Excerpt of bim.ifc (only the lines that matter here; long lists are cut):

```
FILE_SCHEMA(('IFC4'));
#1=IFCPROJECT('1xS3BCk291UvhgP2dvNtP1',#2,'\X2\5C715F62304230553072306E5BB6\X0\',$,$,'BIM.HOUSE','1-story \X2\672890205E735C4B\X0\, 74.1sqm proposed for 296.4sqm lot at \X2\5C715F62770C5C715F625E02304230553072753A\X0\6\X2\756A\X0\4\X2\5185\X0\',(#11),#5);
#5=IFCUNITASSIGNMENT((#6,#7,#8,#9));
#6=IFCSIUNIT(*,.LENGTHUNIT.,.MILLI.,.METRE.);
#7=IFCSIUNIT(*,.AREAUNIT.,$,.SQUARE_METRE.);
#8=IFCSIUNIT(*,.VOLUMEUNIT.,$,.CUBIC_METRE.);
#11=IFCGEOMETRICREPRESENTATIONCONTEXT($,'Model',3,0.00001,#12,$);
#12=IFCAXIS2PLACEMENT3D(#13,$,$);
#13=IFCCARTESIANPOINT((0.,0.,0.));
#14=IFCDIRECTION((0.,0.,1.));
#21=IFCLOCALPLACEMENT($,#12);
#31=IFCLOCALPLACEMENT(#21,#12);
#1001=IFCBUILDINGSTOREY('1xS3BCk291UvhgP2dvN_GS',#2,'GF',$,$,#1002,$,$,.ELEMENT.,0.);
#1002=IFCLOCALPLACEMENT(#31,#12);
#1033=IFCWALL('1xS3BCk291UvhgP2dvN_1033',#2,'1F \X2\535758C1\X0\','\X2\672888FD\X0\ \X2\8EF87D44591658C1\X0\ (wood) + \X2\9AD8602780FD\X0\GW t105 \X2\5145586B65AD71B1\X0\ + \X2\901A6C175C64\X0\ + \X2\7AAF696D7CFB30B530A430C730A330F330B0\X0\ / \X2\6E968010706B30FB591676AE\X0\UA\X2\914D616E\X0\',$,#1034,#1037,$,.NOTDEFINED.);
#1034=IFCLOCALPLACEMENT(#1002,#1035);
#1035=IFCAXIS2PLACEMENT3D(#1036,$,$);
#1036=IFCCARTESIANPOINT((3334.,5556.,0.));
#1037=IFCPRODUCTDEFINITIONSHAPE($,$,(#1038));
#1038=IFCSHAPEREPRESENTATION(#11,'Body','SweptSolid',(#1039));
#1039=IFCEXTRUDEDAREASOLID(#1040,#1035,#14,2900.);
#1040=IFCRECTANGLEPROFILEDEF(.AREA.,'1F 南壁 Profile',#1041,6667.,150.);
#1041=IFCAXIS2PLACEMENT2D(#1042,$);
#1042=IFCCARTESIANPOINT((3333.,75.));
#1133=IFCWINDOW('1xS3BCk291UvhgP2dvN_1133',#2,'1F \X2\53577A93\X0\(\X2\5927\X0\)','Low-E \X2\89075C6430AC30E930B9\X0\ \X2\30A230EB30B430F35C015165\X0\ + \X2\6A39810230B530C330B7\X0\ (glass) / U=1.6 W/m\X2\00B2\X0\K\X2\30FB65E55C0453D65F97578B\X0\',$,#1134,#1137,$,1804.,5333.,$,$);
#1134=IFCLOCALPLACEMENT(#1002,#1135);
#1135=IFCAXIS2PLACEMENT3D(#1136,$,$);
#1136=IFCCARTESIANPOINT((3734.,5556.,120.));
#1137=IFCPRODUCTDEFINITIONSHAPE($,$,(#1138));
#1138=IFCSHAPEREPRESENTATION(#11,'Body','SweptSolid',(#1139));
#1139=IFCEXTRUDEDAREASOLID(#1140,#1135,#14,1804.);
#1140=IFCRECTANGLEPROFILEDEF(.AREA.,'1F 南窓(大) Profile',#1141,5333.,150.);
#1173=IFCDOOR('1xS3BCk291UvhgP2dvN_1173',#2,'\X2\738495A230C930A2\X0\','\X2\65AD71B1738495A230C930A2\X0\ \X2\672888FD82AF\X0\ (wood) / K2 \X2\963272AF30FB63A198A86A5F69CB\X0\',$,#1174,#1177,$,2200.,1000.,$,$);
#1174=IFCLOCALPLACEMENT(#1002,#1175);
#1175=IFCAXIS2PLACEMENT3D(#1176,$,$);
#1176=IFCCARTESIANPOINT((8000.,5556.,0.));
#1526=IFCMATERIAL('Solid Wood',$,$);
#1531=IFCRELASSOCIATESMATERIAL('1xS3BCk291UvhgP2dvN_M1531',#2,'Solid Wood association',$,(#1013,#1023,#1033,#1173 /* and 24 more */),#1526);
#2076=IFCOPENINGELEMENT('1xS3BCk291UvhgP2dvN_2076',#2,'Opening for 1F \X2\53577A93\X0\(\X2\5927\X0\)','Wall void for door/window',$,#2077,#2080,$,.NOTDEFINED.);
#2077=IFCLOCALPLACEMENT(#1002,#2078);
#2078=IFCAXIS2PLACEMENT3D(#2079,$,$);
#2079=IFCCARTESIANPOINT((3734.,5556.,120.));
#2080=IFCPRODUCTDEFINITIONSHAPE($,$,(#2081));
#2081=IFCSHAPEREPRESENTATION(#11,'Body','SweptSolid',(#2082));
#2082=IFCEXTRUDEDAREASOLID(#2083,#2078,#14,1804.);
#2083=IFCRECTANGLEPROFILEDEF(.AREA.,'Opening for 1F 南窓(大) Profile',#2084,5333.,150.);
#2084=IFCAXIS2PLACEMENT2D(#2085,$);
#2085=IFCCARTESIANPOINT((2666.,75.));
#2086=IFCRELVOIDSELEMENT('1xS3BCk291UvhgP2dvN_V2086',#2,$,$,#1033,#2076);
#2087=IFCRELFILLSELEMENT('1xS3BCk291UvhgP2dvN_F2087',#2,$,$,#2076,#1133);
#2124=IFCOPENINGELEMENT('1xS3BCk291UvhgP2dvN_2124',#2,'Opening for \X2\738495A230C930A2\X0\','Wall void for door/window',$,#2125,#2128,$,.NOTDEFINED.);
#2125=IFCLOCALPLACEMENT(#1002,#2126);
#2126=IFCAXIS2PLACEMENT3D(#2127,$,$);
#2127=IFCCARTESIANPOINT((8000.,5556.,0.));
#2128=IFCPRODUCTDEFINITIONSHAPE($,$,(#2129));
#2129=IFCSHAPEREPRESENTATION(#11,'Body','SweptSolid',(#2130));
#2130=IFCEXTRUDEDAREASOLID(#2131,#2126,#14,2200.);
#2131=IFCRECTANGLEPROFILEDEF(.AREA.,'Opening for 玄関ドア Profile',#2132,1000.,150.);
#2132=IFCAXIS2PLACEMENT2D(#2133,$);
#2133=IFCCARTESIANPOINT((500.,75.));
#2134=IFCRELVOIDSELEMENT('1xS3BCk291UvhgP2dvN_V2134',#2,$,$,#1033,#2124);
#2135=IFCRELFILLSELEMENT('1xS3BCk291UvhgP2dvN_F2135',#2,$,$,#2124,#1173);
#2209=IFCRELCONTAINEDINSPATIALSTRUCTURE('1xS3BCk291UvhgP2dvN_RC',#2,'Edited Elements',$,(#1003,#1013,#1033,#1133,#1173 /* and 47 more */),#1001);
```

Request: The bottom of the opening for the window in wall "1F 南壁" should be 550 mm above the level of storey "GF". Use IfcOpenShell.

```python
import numpy as np
import ifcopenshell
import ifcopenshell.api.geometry
import ifcopenshell.geom
import ifcopenshell.util.element
import ifcopenshell.util.placement
import ifcopenshell.util.shape
import ifcopenshell.util.unit

model = ifcopenshell.open("bim.ifc")
unit_scale = ifcopenshell.util.unit.calculate_unit_scale(model)

window = model.by_id(1133)
opening = window.FillsVoids[0].RelatingOpeningElement
storey = ifcopenshell.util.element.get_container(window, ifc_class="IfcBuildingStorey")
level = ifcopenshell.util.placement.get_local_placement(storey.ObjectPlacement)[2, 3]

# The opening's origin need not be at the sill, so measure its lowest point.
shape = ifcopenshell.geom.create_shape(ifcopenshell.geom.settings(), opening)
bottom = ifcopenshell.util.shape.get_shape_bottom_elevation(shape, shape.geometry) / unit_scale
dz = level + 550.0 - bottom

shift = np.array([0.0, 0.0, dz])
# The window is not placed relative to its opening, so move both.
for product in (opening, window):
    matrix = ifcopenshell.util.placement.get_local_placement(product.ObjectPlacement)
    matrix[:3, 3] += shift
    ifcopenshell.api.geometry.edit_object_placement(model, product=product, matrix=matrix, is_si=False)

print(f"moved by {dz * unit_scale:+.3f} m")

model.write("bim_rev.ifc")
```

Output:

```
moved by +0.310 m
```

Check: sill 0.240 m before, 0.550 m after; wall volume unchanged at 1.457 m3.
